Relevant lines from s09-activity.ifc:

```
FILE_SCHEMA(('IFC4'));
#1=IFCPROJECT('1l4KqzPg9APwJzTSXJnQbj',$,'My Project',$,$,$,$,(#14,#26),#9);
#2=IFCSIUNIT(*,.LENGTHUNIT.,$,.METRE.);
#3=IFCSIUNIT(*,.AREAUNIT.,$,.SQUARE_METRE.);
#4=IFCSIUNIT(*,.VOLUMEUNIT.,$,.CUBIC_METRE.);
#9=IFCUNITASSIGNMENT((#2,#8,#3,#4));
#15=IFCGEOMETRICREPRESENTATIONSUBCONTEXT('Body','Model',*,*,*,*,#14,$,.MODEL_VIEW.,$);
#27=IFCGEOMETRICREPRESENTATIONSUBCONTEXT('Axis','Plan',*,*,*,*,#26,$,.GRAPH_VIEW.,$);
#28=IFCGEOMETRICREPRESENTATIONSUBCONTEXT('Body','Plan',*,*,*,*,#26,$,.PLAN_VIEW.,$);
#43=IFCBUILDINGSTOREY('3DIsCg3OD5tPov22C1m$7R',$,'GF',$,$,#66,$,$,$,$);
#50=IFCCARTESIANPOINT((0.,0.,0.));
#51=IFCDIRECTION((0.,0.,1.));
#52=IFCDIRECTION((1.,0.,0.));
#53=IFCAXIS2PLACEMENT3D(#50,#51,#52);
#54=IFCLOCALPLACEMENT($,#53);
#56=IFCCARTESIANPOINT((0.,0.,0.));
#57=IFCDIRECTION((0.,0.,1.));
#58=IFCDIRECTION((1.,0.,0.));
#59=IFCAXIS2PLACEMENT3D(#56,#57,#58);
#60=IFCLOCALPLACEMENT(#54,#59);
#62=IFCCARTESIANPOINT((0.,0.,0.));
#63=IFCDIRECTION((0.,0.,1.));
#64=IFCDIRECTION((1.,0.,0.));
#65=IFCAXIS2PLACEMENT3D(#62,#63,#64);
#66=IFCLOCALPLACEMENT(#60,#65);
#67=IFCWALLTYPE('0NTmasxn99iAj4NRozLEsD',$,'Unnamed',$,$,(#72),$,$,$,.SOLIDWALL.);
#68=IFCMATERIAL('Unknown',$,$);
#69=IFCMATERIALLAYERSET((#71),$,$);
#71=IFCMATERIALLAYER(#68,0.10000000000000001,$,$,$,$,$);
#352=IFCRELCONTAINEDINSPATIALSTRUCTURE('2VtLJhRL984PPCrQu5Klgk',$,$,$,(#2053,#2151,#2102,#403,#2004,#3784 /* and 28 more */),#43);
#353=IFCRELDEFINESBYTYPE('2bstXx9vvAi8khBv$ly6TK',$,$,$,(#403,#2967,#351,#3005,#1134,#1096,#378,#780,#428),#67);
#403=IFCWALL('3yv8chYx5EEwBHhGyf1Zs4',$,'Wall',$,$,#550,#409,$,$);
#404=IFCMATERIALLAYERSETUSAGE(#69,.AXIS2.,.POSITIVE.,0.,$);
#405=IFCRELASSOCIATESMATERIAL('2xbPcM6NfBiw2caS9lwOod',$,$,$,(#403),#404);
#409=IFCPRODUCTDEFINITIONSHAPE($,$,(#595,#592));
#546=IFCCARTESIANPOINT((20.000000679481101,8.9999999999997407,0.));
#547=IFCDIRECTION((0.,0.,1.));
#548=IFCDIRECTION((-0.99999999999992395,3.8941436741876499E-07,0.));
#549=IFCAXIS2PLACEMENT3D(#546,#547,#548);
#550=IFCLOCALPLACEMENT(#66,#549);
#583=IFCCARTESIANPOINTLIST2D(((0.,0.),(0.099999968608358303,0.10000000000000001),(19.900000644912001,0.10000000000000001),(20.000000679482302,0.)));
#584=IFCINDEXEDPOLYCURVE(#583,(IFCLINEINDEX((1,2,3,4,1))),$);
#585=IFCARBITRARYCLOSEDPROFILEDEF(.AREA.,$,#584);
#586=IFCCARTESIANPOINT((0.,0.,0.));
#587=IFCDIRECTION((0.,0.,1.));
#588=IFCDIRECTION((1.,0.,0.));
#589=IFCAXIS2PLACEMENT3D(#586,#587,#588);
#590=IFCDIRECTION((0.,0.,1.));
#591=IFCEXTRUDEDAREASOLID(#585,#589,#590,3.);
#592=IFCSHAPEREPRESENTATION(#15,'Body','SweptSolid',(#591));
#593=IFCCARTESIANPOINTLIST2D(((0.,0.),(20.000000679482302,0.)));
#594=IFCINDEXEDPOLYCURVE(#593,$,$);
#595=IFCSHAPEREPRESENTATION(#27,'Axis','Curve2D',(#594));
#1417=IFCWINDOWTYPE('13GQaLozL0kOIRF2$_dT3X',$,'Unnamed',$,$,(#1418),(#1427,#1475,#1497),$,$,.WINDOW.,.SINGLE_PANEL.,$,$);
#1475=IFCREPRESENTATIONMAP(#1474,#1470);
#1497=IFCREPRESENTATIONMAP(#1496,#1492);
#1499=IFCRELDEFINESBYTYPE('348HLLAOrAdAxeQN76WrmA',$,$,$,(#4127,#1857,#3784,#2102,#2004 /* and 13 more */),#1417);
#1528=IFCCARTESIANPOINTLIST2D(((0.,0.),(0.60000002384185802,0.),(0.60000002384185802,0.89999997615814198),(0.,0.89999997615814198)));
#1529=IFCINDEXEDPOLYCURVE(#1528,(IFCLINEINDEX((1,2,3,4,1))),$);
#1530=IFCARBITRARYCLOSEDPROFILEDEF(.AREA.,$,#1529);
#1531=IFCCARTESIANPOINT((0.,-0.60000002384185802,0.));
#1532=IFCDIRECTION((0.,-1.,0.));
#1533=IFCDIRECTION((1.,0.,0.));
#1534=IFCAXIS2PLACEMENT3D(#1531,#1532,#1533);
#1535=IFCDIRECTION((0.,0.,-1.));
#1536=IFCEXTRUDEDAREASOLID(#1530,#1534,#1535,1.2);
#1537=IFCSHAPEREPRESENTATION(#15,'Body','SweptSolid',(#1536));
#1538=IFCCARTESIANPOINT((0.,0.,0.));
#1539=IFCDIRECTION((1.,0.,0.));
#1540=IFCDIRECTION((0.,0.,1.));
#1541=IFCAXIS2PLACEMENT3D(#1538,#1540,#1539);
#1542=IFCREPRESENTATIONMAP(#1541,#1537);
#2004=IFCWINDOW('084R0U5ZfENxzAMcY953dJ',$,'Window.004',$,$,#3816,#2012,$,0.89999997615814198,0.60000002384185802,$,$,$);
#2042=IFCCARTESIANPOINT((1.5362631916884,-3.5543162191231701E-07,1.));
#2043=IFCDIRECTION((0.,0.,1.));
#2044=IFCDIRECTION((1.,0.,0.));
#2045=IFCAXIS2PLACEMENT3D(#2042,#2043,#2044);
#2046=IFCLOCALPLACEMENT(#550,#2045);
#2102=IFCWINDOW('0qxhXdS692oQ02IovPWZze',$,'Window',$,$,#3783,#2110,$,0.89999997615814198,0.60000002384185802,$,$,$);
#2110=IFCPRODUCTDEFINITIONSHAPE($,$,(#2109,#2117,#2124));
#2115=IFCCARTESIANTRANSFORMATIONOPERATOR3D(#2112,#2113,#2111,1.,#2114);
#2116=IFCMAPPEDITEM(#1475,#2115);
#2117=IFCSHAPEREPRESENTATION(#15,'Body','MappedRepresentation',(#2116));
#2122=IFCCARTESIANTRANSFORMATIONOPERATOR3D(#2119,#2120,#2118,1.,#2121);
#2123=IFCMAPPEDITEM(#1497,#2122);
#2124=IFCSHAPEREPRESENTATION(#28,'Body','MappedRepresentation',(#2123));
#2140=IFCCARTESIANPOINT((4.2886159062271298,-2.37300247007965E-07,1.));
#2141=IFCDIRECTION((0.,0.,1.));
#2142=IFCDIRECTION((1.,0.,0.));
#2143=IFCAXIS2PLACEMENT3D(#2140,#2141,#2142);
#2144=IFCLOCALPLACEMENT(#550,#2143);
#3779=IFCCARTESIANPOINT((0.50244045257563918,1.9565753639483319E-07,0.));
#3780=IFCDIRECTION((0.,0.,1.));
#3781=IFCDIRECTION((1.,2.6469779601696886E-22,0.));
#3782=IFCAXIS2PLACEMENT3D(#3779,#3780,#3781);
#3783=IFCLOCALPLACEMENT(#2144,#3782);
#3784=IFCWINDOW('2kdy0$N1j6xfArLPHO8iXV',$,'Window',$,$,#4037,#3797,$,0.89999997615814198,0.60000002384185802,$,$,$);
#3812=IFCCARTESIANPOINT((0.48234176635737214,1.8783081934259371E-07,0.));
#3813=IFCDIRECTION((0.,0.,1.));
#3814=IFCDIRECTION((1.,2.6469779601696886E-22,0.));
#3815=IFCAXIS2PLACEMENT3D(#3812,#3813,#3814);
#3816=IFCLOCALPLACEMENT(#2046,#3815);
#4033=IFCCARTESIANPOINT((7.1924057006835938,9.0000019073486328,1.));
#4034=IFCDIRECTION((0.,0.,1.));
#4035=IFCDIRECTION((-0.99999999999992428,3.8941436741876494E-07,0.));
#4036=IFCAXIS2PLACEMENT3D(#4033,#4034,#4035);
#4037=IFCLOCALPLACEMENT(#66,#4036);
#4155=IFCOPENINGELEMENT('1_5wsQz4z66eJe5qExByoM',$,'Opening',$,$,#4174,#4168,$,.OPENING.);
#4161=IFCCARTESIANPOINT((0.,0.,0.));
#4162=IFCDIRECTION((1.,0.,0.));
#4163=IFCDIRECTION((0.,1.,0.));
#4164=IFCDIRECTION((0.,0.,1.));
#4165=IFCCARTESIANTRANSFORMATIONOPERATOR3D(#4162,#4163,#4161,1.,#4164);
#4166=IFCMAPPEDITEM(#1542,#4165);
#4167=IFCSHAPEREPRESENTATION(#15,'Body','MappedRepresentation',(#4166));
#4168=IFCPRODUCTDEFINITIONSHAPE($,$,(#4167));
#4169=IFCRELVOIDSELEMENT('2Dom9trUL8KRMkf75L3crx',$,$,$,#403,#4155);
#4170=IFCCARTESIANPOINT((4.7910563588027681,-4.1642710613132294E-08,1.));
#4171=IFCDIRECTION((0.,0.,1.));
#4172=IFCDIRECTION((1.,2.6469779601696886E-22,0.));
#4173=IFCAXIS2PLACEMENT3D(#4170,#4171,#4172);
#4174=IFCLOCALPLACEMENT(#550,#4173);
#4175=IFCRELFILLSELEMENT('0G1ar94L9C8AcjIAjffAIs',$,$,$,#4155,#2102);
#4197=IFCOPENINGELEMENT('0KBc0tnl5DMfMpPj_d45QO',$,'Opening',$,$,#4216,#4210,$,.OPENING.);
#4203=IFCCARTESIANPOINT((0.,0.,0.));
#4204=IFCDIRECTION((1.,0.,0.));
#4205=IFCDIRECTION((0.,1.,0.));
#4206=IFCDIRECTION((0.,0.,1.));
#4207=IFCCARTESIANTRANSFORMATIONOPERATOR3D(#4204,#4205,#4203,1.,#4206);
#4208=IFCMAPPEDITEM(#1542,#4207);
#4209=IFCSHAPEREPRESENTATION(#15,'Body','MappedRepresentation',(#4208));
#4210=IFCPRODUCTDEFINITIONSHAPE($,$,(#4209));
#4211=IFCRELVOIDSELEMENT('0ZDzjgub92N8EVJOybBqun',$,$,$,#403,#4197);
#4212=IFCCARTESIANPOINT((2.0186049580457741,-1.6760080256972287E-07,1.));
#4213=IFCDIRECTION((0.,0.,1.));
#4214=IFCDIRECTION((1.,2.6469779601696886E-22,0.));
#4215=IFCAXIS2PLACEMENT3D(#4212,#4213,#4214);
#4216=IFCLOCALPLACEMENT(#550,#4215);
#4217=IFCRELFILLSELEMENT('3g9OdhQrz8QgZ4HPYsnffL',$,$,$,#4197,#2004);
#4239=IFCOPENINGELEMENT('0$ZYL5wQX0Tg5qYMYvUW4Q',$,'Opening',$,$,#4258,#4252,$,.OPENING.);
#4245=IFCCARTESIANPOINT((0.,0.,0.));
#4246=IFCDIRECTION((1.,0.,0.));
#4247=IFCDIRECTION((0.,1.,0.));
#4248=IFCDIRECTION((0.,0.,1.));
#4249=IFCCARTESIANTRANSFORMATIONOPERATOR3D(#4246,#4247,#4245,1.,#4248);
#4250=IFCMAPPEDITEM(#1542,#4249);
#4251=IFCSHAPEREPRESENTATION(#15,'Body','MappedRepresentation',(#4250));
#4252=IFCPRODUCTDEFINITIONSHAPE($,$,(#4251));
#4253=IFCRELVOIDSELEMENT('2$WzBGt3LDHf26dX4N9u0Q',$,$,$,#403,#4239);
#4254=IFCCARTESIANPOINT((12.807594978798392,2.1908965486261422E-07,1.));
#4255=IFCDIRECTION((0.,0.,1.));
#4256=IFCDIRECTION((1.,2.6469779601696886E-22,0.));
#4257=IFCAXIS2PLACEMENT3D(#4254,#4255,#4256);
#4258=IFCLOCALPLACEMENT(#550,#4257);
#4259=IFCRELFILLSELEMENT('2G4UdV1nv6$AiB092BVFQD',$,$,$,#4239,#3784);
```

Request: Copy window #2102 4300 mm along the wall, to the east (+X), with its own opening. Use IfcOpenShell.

```python
import ifcopenshell
import ifcopenshell.api.feature
import ifcopenshell.api.geometry
import ifcopenshell.api.root
import ifcopenshell.geom
import ifcopenshell.util.element
import ifcopenshell.util.placement
import ifcopenshell.util.shape
import ifcopenshell.util.unit

model = ifcopenshell.open("s09-activity.ifc")
unit_scale = ifcopenshell.util.unit.calculate_unit_scale(model)
settings = ifcopenshell.geom.settings()


def volume(element):
    """Net volume in cubic metres, openings subtracted."""
    shape = ifcopenshell.geom.create_shape(settings, element)
    return ifcopenshell.util.shape.get_volume(shape.geometry)


window = model.by_guid("0qxhXdS692oQ02IovPWZze")
opening = window.FillsVoids[0].RelatingOpeningElement
wall = opening.VoidsElements[0].RelatingBuildingElement
before = volume(wall)
shift = ifcopenshell.util.placement.get_local_placement(wall.ObjectPlacement)[:3, 0] * -4.3 / unit_scale

# copy_class copies the void relationship, type, container and properties, but no geometry.
new_opening = ifcopenshell.api.root.copy_class(model, product=opening)
new_opening.Representation = ifcopenshell.util.element.copy_deep(
    model, opening.Representation, exclude=["IfcGeometricRepresentationContext", "IfcRepresentationMap"]
)
new_window = ifcopenshell.api.root.copy_class(model, product=window)
new_window.Representation = ifcopenshell.util.element.copy_deep(
    model, window.Representation, exclude=["IfcGeometricRepresentationContext", "IfcRepresentationMap"]
)
ifcopenshell.api.feature.add_filling(model, opening=new_opening, element=new_window)

for old, new in ((opening, new_opening), (window, new_window)):
    matrix = ifcopenshell.util.placement.get_local_placement(old.ObjectPlacement)
    matrix[:3, 3] += shift
    ifcopenshell.api.geometry.edit_object_placement(model, product=new, matrix=matrix, is_si=False)

after = volume(wall)

print(f"wall volume {before:.3f} -> {after:.3f} m3")

model.write("s09-activity_v2.ifc")
```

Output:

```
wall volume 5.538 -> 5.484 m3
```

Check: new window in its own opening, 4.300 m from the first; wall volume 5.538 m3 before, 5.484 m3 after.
